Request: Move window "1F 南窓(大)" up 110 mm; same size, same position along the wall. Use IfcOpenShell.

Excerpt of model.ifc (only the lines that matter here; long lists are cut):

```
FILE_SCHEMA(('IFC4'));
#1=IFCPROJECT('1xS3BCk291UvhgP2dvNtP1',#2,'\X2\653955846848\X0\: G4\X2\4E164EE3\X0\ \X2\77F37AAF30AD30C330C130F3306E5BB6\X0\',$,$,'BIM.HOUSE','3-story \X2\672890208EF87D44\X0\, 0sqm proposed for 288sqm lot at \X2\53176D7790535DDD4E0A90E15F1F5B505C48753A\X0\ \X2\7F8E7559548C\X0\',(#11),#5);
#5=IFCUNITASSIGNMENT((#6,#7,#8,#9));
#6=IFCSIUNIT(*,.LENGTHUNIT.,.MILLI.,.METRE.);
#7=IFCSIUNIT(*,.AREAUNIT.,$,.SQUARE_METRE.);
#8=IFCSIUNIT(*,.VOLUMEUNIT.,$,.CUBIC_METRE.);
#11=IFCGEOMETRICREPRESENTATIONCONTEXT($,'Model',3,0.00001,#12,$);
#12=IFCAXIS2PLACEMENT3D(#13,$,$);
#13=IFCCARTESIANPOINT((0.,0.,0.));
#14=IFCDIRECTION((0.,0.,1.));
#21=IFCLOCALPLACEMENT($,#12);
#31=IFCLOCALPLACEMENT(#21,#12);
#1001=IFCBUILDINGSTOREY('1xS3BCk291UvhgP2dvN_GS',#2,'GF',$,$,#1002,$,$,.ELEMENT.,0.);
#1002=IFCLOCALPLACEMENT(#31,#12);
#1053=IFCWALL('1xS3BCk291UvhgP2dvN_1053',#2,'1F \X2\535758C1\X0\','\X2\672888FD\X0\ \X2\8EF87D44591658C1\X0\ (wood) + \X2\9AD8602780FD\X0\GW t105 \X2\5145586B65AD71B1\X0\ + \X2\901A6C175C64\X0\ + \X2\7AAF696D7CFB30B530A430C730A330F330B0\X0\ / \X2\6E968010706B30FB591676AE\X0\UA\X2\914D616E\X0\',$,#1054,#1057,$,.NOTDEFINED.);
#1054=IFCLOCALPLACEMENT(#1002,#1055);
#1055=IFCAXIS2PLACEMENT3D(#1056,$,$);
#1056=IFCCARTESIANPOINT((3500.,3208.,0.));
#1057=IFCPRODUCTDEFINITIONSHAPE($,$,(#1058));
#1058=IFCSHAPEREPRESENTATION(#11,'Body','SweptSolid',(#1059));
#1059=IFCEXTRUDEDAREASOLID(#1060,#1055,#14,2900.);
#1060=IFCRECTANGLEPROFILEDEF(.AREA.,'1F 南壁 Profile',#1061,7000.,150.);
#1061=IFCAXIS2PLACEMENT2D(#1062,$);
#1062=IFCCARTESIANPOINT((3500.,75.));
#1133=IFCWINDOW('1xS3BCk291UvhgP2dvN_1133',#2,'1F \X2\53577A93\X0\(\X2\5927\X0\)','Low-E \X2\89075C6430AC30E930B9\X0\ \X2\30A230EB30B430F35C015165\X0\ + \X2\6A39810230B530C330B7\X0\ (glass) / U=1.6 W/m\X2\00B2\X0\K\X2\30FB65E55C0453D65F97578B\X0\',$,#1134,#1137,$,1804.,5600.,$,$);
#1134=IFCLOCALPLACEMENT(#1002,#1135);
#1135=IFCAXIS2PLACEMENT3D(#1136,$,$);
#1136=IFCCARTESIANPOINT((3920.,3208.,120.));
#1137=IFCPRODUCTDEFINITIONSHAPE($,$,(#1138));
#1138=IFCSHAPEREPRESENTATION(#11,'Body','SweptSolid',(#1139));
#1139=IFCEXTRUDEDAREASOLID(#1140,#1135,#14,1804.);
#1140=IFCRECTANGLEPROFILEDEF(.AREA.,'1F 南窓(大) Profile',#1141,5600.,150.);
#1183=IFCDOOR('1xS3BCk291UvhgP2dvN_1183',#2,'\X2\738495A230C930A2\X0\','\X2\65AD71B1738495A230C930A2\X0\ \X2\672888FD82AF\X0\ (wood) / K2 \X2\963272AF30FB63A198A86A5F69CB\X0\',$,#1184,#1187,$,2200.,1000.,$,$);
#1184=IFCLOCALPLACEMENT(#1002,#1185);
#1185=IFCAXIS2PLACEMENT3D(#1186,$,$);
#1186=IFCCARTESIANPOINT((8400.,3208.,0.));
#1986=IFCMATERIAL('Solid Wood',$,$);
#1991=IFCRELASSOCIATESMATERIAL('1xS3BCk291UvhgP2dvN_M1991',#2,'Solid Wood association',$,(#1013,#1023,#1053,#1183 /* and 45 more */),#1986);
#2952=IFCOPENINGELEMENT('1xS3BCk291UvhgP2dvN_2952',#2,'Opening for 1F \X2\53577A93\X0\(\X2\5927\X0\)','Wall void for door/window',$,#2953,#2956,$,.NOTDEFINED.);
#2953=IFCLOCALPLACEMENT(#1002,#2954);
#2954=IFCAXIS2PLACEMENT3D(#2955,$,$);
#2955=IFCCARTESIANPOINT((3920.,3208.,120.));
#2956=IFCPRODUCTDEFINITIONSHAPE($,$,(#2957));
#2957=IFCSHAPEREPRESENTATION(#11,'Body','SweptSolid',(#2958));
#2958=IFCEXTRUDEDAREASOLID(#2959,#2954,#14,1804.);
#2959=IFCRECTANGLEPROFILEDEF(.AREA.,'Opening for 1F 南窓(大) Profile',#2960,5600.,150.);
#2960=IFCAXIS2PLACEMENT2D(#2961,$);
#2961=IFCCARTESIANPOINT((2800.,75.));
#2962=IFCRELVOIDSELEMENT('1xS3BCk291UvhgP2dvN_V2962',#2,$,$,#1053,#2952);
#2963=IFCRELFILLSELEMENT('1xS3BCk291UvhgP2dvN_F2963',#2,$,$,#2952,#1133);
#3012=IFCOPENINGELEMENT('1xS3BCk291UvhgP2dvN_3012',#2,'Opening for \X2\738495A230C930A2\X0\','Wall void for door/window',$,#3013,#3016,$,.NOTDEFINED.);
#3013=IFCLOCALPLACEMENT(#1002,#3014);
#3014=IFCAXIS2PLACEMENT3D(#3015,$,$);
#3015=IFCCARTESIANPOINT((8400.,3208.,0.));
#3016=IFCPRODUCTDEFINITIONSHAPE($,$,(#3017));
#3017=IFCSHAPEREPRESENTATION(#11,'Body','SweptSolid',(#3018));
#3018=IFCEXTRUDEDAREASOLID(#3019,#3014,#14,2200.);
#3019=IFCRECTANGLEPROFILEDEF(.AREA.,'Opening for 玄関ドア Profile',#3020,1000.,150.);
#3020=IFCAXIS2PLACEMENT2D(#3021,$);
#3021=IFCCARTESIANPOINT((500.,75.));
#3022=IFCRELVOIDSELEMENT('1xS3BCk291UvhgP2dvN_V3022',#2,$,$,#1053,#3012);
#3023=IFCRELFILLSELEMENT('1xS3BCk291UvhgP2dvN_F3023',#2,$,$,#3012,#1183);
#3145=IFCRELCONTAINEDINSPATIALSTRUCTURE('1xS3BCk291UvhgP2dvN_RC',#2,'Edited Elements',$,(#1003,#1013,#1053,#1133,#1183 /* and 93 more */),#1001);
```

```python
import numpy as np
import ifcopenshell
import ifcopenshell.api.geometry
import ifcopenshell.util.placement
import ifcopenshell.util.unit

model = ifcopenshell.open("model.ifc")
unit_scale = ifcopenshell.util.unit.calculate_unit_scale(model)

window = model.by_guid("1xS3BCk291UvhgP2dvN_1133")
opening = window.FillsVoids[0].RelatingOpeningElement
dz = 110.0

shift = np.array([0.0, 0.0, dz])
# The window is not placed relative to its opening, so move both.
for product in (opening, window):
    matrix = ifcopenshell.util.placement.get_local_placement(product.ObjectPlacement)
    matrix[:3, 3] += shift
    ifcopenshell.api.geometry.edit_object_placement(model, product=product, matrix=matrix, is_si=False)

print(f"moved by {dz * unit_scale:+.3f} m")

model.write("model_updated.ifc")
```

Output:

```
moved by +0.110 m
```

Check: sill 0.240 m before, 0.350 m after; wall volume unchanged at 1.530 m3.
